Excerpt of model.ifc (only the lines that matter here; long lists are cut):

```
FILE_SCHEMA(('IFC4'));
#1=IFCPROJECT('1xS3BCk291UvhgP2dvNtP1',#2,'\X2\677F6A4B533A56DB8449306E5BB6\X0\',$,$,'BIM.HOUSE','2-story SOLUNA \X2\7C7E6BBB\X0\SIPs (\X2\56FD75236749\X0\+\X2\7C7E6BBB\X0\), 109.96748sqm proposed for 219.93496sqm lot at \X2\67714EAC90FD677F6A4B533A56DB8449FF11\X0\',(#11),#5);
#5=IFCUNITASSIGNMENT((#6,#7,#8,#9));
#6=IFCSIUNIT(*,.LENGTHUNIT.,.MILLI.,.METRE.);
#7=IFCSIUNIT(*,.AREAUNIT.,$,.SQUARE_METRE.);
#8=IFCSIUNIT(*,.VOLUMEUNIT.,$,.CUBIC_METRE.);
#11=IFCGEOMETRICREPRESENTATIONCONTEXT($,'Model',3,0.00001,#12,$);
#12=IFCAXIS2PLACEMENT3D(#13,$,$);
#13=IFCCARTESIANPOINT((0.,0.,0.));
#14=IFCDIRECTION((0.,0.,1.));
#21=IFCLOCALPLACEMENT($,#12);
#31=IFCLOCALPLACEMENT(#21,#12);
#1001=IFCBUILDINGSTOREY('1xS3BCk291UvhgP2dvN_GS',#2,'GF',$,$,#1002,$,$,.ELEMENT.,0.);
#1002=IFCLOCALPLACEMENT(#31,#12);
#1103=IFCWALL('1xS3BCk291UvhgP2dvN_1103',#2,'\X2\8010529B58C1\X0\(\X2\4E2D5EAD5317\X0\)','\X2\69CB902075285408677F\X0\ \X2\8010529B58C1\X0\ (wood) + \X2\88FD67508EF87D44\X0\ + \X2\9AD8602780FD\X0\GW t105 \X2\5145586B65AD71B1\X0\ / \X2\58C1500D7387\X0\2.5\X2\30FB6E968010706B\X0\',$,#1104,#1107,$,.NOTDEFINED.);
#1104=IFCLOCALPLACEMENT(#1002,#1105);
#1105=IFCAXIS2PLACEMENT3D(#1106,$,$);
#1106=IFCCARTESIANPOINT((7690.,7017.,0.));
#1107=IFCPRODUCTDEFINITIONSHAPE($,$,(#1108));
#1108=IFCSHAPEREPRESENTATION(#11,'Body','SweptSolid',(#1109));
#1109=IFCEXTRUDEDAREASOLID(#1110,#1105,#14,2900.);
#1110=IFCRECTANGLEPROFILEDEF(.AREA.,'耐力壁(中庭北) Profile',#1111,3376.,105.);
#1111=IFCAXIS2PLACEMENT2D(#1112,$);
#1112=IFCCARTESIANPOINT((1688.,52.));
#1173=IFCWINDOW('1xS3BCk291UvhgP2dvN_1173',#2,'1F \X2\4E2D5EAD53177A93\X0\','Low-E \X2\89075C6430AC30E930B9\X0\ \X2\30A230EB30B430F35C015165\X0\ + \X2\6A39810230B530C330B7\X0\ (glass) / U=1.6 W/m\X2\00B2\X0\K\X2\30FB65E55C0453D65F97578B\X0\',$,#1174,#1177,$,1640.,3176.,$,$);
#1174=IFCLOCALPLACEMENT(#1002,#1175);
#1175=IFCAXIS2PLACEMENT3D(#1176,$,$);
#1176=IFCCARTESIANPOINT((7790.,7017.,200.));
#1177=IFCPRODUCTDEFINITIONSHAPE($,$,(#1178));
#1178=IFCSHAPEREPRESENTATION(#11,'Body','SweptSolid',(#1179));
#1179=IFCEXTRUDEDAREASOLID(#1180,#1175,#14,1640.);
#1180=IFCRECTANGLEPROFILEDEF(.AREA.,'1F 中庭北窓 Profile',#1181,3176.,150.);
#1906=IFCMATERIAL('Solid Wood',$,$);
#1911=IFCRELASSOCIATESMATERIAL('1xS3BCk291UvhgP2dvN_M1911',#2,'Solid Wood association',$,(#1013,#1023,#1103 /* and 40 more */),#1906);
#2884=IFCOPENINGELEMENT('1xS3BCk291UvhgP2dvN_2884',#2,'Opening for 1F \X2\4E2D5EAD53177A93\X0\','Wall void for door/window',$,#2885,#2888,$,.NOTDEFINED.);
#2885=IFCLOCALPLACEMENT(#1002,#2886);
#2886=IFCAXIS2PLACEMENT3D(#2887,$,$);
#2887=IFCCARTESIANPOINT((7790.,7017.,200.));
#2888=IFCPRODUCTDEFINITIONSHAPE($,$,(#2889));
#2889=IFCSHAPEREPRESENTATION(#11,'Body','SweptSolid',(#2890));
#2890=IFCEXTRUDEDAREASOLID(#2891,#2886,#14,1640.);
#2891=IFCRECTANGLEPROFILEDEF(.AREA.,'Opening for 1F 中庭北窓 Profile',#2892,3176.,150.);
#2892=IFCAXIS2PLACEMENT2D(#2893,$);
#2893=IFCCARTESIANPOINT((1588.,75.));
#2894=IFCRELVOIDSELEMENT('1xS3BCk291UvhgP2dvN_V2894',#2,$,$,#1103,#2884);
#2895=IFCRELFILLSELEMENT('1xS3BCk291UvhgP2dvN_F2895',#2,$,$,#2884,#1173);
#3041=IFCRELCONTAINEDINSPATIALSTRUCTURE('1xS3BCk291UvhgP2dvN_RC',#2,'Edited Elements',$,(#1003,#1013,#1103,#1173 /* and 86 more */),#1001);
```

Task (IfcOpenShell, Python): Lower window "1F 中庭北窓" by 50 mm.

```python
import numpy as np
import ifcopenshell
import ifcopenshell.api.geometry
import ifcopenshell.util.placement
import ifcopenshell.util.unit

model = ifcopenshell.open("model.ifc")
unit_scale = ifcopenshell.util.unit.calculate_unit_scale(model)

window = model.by_id(1173)
opening = window.FillsVoids[0].RelatingOpeningElement
dz = -0.05 / unit_scale

shift = np.array([0.0, 0.0, dz])
# The window is not placed relative to its opening, so move both.
for product in (opening, window):
    matrix = ifcopenshell.util.placement.get_local_placement(product.ObjectPlacement)
    matrix[:3, 3] += shift
    ifcopenshell.api.geometry.edit_object_placement(model, product=product, matrix=matrix, is_si=False)

print(f"moved by {dz * unit_scale:+.3f} m")

model.write("model_updated.ifc")
```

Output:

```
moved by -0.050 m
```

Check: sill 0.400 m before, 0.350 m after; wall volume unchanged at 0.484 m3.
